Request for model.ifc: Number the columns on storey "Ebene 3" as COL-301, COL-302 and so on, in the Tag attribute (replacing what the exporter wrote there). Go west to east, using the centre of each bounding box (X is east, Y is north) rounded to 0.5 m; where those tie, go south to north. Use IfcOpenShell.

First a look at what the model holds.

```python
import ifcopenshell
import ifcopenshell.util.element
import ifcopenshell.util.placement

model = ifcopenshell.open("model.ifc")
print(model.schema)
storey = next(s for s in model.by_type("IfcBuildingStorey") if s.Name == "Ebene 3")
columns = [e for e in ifcopenshell.util.element.get_decomposition(storey) if e.is_a("IfcColumn")]
for e in sorted(columns, key=lambda e: e.id()):
    origin = ifcopenshell.util.placement.get_local_placement(e.ObjectPlacement)[:3, 3]
    print(e.id(), e.Tag, e.Name, origin.round(2) + 0.0, sep=" | ")
```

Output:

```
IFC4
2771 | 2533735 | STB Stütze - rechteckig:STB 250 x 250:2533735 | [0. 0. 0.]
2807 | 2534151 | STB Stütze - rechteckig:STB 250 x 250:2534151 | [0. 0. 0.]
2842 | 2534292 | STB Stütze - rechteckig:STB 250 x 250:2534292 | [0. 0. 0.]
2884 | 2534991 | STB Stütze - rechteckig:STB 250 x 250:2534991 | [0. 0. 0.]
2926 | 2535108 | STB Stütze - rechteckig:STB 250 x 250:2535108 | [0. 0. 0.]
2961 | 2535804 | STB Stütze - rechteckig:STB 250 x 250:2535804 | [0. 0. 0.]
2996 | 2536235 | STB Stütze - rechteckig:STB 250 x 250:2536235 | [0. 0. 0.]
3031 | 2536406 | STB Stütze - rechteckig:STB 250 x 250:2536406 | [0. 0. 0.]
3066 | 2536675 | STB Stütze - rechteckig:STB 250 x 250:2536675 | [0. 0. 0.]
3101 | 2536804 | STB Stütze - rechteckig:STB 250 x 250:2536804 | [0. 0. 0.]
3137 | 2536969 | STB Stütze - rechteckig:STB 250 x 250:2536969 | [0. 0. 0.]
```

```python
import ifcopenshell
import ifcopenshell.geom
import ifcopenshell.util.element
import ifcopenshell.util.shape

model = ifcopenshell.open("model.ifc")
settings = ifcopenshell.geom.settings()
settings.set("use-world-coords", True)


def centre(element):
    shape = ifcopenshell.geom.create_shape(settings, element)
    return ifcopenshell.util.shape.get_bbox_centroid(shape.geometry)


storey = next(s for s in model.by_type("IfcBuildingStorey") if s.Name == "Ebene 3")
columns = [e for e in ifcopenshell.util.element.get_decomposition(storey) if e.is_a("IfcColumn")]

# Insertion points can sit at a corner or the storey origin, so sort by the geometry (in metres).
centres = {e: centre(e) for e in columns}
columns.sort(key=lambda e: (round(centres[e][0] / 0.5), centres[e][1]))

for i, e in enumerate(columns, start=1):
    number = f"COL-3{i:02d}"
    e.Tag = number
    print(e.id(), number)

model.write("model_edited.ifc")
```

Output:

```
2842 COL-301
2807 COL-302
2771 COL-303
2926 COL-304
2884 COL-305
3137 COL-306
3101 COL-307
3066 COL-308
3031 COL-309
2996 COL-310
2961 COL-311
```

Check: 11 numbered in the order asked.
